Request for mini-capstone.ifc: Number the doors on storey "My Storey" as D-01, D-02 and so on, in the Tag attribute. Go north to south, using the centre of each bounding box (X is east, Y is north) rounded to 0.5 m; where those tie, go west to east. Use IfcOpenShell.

First a look at what the model holds.

```python
import ifcopenshell
import ifcopenshell.util.element
import ifcopenshell.util.placement

model = ifcopenshell.open("mini-capstone.ifc")
print(model.schema)
storey = next(s for s in model.by_type("IfcBuildingStorey") if s.Name == "My Storey")
doors = [e for e in ifcopenshell.util.element.get_decomposition(storey) if e.is_a("IfcDoor")]
for e in sorted(doors, key=lambda e: e.id()):
    origin = ifcopenshell.util.placement.get_local_placement(e.ObjectPlacement)[:3, 3]
    print(e.id(), e.Tag, e.Name, origin.round(2) + 0.0, sep=" | ")
```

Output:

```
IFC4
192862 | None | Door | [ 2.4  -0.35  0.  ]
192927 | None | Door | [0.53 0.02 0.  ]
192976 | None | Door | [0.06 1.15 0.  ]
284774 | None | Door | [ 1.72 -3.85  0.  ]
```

```python
import ifcopenshell
import ifcopenshell.geom
import ifcopenshell.util.element
import ifcopenshell.util.shape

model = ifcopenshell.open("mini-capstone.ifc")
settings = ifcopenshell.geom.settings()
settings.set("use-world-coords", True)


def centre(element):
    shape = ifcopenshell.geom.create_shape(settings, element)
    return ifcopenshell.util.shape.get_bbox_centroid(shape.geometry)


storey = next(s for s in model.by_type("IfcBuildingStorey") if s.Name == "My Storey")
doors = [e for e in ifcopenshell.util.element.get_decomposition(storey) if e.is_a("IfcDoor")]

# Insertion points can sit at a corner or the storey origin, so sort by the geometry (in metres).
centres = {e: centre(e) for e in doors}
doors.sort(key=lambda e: (-round(centres[e][1] / 0.5), centres[e][0]))

for i, e in enumerate(doors, start=1):
    number = f"D-{i:02d}"
    e.Tag = number
    print(e.id(), number)

model.write("mini-capstone_updated.ifc")
```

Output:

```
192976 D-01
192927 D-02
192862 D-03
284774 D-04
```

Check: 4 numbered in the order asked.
